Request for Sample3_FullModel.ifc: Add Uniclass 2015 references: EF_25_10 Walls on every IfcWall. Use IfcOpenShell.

First a look at what the model holds.

```python
import ifcopenshell

model = ifcopenshell.open("Sample3_FullModel.ifc")
print(model.schema)
print("classifications:", [c.Name for c in model.by_type("IfcClassification")])
for ifc_class in ("IfcDoor", "IfcRoof", "IfcStair", "IfcWall", "IfcWindow"):
    print(ifc_class, len(model.by_type(ifc_class)))
```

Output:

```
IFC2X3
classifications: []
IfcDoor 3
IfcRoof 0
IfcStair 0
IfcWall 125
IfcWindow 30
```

```python
import ifcopenshell
import ifcopenshell.api.classification

model = ifcopenshell.open("Sample3_FullModel.ifc")

# IFC2X3 requires Source and Edition and has no link from the project to the system.
system = model.create_entity("IfcClassification", Source="NBS", Edition="2015", Name="Uniclass 2015")

codes = {
    "IfcWall": ("EF_25_10", "Walls"),
}
for ifc_class, (code, name) in codes.items():
    products = model.by_type(ifc_class)
    ifcopenshell.api.classification.add_reference(
        model, products=products, classification=system, identification=code, name=name
    )
    print(code, len(products))

model.write("Sample3_FullModel_updated.ifc")
```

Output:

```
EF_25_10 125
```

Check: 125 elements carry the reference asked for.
